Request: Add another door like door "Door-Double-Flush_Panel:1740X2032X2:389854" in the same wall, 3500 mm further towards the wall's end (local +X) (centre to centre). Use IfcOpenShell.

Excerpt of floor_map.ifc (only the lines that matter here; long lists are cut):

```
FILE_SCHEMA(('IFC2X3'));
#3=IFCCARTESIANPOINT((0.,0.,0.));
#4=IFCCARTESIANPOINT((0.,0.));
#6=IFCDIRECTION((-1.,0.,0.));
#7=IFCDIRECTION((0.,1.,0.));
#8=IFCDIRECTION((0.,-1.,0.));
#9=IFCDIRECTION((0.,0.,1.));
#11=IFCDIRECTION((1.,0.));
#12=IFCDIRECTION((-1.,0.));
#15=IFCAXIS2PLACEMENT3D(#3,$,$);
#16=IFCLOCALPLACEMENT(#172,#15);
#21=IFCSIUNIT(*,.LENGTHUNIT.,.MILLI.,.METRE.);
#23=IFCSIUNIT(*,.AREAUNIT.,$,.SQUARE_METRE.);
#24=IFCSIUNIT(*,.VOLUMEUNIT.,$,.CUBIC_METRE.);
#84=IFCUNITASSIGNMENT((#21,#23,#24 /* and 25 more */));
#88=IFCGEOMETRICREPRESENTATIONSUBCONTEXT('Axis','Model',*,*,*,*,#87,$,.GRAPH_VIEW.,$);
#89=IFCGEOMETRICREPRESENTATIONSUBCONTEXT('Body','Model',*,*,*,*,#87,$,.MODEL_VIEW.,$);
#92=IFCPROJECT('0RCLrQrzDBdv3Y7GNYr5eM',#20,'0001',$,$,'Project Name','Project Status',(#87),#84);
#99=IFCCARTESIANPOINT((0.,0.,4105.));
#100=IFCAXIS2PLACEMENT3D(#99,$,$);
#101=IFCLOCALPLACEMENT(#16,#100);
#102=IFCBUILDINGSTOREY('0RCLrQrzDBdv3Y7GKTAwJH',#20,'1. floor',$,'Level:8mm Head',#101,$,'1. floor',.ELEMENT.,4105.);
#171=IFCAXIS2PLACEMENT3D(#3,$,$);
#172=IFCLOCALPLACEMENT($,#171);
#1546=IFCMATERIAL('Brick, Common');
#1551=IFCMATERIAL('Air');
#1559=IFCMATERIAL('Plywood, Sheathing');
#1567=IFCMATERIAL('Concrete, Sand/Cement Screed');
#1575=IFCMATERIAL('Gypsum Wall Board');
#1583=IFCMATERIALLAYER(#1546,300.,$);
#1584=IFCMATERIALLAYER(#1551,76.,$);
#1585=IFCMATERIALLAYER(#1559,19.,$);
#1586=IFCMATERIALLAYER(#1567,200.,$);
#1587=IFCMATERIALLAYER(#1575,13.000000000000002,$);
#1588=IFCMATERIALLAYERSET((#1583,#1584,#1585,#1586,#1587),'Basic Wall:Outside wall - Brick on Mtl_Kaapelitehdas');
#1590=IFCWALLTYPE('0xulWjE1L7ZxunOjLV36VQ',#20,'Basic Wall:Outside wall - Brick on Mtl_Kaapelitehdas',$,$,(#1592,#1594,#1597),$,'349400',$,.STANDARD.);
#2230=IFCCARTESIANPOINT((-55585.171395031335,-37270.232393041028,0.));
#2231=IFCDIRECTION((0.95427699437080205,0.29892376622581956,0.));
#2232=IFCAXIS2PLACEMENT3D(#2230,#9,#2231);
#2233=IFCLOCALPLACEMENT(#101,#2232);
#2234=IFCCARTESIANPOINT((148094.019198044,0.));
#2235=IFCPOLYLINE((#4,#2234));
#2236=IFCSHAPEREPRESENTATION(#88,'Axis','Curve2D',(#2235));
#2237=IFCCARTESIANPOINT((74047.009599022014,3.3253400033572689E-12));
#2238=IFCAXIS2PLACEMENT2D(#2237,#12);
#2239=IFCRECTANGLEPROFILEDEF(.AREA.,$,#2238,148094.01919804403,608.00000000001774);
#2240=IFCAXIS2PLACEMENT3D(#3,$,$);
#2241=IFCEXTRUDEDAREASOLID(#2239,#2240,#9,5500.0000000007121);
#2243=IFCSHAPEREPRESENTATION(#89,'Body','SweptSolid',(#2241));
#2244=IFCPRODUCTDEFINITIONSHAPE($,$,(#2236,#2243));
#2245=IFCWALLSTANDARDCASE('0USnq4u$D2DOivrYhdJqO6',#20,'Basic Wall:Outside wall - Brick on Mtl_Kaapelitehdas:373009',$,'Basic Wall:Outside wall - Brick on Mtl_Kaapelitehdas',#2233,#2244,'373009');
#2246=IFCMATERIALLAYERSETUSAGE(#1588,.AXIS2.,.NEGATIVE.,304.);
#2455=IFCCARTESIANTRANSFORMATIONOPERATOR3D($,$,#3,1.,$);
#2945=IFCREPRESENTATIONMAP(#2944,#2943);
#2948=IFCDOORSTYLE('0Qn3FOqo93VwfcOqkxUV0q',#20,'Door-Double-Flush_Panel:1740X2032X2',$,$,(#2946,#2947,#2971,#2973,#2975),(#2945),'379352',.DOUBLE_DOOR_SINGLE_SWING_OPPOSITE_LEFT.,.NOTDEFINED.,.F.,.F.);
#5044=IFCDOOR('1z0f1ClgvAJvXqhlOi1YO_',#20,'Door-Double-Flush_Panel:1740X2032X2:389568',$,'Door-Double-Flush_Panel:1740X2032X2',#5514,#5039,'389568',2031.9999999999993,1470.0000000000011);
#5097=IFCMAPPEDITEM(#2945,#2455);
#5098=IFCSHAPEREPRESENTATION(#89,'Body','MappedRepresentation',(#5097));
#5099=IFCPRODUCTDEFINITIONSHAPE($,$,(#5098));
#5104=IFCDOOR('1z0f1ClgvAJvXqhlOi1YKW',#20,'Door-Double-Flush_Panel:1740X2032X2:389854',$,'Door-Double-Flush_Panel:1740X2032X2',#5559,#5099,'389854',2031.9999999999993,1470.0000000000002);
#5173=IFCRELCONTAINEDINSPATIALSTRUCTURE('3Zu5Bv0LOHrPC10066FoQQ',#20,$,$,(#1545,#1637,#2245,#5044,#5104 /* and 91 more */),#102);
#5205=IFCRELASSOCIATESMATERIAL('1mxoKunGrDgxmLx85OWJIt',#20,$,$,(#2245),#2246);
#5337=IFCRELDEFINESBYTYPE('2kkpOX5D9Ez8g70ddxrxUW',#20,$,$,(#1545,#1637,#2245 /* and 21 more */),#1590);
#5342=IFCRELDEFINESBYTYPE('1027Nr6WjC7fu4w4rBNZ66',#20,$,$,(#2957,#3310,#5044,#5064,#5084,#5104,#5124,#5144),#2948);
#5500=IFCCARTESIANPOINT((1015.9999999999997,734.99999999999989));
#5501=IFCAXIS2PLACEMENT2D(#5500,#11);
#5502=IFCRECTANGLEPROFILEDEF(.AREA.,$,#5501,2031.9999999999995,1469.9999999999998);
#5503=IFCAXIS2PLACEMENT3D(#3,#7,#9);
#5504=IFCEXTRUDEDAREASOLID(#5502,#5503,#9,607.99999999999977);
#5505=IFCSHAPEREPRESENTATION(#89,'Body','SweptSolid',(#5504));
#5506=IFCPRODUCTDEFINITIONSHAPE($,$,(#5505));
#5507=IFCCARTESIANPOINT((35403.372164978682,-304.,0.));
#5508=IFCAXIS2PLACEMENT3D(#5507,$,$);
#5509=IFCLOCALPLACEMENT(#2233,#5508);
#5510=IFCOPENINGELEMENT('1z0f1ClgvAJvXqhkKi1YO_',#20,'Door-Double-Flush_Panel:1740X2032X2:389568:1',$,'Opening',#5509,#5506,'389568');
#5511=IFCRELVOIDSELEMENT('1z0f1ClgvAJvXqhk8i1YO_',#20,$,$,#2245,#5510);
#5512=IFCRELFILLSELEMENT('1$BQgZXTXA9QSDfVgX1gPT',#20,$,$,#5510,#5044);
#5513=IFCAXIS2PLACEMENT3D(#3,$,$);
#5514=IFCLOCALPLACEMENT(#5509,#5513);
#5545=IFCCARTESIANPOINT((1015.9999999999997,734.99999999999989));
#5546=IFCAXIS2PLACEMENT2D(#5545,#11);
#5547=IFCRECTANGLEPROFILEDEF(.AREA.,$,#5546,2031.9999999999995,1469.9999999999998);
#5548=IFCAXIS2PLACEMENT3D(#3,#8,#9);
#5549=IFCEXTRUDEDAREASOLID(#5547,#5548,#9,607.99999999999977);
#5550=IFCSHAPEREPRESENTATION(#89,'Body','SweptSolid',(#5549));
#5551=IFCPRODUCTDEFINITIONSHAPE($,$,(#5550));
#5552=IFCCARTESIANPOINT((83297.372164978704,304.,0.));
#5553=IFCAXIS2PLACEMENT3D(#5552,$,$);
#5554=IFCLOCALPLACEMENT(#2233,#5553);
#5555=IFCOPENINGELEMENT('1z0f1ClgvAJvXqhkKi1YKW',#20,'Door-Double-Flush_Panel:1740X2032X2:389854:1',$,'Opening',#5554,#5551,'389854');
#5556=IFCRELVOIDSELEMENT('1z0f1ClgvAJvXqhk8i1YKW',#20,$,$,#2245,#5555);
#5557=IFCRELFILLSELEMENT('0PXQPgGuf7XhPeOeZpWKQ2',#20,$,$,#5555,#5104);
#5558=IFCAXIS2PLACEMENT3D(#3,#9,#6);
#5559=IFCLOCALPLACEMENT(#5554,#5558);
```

```python
import ifcopenshell
import ifcopenshell.api.feature
import ifcopenshell.api.geometry
import ifcopenshell.api.root
import ifcopenshell.geom
import ifcopenshell.util.element
import ifcopenshell.util.placement
import ifcopenshell.util.shape
import ifcopenshell.util.unit

model = ifcopenshell.open("floor_map.ifc")
unit_scale = ifcopenshell.util.unit.calculate_unit_scale(model)
settings = ifcopenshell.geom.settings()


def volume(element):
    """Net volume in cubic metres, openings subtracted."""
    shape = ifcopenshell.geom.create_shape(settings, element)
    return ifcopenshell.util.shape.get_volume(shape.geometry)


def reuse_history(source, copy):
    """copy_class also copies each property set's owner history, people and application; keep the originals."""
    for rel in copy.IsDefinedBy:
        if rel.is_a("IfcRelDefinesByProperties") and (history := rel.RelatingPropertyDefinition.OwnerHistory):
            rel.RelatingPropertyDefinition.OwnerHistory = source.OwnerHistory
            ifcopenshell.util.element.remove_deep2(model, history)


door = model.by_id(5104)
opening = door.FillsVoids[0].RelatingOpeningElement
wall = opening.VoidsElements[0].RelatingBuildingElement
before = volume(wall)
shift = ifcopenshell.util.placement.get_local_placement(wall.ObjectPlacement)[:3, 0] * 3.5 / unit_scale

# copy_class copies the void relationship, type, container and properties, but no geometry.
new_opening = ifcopenshell.api.root.copy_class(model, product=opening)
new_opening.Representation = ifcopenshell.util.element.copy_deep(
    model, opening.Representation, exclude=["IfcGeometricRepresentationContext", "IfcRepresentationMap"]
)
new_opening.Name = "Door-Double-Flush_Panel:1740X2032X2"
new_opening.Tag = None
new_door = ifcopenshell.api.root.copy_class(model, product=door)
new_door.Representation = ifcopenshell.util.element.copy_deep(
    model, door.Representation, exclude=["IfcGeometricRepresentationContext", "IfcRepresentationMap"]
)
new_door.Name = "Door-Double-Flush_Panel:1740X2032X2"
new_door.Tag = None
reuse_history(door, new_door)
fills = ifcopenshell.api.feature.add_filling(model, opening=new_opening, element=new_door)
fills.OwnerHistory = new_door.OwnerHistory  # required in IFC2X3

for old, new in ((opening, new_opening), (door, new_door)):
    matrix = ifcopenshell.util.placement.get_local_placement(old.ObjectPlacement)
    matrix[:3, 3] += shift
    ifcopenshell.api.geometry.edit_object_placement(model, product=new, matrix=matrix, is_si=False)

after = volume(wall)

print(f"wall volume {before:.3f} -> {after:.3f} m3")

model.write("floor_map-out.ifc")
```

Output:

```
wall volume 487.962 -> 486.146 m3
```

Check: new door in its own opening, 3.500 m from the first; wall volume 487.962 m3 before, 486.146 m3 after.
